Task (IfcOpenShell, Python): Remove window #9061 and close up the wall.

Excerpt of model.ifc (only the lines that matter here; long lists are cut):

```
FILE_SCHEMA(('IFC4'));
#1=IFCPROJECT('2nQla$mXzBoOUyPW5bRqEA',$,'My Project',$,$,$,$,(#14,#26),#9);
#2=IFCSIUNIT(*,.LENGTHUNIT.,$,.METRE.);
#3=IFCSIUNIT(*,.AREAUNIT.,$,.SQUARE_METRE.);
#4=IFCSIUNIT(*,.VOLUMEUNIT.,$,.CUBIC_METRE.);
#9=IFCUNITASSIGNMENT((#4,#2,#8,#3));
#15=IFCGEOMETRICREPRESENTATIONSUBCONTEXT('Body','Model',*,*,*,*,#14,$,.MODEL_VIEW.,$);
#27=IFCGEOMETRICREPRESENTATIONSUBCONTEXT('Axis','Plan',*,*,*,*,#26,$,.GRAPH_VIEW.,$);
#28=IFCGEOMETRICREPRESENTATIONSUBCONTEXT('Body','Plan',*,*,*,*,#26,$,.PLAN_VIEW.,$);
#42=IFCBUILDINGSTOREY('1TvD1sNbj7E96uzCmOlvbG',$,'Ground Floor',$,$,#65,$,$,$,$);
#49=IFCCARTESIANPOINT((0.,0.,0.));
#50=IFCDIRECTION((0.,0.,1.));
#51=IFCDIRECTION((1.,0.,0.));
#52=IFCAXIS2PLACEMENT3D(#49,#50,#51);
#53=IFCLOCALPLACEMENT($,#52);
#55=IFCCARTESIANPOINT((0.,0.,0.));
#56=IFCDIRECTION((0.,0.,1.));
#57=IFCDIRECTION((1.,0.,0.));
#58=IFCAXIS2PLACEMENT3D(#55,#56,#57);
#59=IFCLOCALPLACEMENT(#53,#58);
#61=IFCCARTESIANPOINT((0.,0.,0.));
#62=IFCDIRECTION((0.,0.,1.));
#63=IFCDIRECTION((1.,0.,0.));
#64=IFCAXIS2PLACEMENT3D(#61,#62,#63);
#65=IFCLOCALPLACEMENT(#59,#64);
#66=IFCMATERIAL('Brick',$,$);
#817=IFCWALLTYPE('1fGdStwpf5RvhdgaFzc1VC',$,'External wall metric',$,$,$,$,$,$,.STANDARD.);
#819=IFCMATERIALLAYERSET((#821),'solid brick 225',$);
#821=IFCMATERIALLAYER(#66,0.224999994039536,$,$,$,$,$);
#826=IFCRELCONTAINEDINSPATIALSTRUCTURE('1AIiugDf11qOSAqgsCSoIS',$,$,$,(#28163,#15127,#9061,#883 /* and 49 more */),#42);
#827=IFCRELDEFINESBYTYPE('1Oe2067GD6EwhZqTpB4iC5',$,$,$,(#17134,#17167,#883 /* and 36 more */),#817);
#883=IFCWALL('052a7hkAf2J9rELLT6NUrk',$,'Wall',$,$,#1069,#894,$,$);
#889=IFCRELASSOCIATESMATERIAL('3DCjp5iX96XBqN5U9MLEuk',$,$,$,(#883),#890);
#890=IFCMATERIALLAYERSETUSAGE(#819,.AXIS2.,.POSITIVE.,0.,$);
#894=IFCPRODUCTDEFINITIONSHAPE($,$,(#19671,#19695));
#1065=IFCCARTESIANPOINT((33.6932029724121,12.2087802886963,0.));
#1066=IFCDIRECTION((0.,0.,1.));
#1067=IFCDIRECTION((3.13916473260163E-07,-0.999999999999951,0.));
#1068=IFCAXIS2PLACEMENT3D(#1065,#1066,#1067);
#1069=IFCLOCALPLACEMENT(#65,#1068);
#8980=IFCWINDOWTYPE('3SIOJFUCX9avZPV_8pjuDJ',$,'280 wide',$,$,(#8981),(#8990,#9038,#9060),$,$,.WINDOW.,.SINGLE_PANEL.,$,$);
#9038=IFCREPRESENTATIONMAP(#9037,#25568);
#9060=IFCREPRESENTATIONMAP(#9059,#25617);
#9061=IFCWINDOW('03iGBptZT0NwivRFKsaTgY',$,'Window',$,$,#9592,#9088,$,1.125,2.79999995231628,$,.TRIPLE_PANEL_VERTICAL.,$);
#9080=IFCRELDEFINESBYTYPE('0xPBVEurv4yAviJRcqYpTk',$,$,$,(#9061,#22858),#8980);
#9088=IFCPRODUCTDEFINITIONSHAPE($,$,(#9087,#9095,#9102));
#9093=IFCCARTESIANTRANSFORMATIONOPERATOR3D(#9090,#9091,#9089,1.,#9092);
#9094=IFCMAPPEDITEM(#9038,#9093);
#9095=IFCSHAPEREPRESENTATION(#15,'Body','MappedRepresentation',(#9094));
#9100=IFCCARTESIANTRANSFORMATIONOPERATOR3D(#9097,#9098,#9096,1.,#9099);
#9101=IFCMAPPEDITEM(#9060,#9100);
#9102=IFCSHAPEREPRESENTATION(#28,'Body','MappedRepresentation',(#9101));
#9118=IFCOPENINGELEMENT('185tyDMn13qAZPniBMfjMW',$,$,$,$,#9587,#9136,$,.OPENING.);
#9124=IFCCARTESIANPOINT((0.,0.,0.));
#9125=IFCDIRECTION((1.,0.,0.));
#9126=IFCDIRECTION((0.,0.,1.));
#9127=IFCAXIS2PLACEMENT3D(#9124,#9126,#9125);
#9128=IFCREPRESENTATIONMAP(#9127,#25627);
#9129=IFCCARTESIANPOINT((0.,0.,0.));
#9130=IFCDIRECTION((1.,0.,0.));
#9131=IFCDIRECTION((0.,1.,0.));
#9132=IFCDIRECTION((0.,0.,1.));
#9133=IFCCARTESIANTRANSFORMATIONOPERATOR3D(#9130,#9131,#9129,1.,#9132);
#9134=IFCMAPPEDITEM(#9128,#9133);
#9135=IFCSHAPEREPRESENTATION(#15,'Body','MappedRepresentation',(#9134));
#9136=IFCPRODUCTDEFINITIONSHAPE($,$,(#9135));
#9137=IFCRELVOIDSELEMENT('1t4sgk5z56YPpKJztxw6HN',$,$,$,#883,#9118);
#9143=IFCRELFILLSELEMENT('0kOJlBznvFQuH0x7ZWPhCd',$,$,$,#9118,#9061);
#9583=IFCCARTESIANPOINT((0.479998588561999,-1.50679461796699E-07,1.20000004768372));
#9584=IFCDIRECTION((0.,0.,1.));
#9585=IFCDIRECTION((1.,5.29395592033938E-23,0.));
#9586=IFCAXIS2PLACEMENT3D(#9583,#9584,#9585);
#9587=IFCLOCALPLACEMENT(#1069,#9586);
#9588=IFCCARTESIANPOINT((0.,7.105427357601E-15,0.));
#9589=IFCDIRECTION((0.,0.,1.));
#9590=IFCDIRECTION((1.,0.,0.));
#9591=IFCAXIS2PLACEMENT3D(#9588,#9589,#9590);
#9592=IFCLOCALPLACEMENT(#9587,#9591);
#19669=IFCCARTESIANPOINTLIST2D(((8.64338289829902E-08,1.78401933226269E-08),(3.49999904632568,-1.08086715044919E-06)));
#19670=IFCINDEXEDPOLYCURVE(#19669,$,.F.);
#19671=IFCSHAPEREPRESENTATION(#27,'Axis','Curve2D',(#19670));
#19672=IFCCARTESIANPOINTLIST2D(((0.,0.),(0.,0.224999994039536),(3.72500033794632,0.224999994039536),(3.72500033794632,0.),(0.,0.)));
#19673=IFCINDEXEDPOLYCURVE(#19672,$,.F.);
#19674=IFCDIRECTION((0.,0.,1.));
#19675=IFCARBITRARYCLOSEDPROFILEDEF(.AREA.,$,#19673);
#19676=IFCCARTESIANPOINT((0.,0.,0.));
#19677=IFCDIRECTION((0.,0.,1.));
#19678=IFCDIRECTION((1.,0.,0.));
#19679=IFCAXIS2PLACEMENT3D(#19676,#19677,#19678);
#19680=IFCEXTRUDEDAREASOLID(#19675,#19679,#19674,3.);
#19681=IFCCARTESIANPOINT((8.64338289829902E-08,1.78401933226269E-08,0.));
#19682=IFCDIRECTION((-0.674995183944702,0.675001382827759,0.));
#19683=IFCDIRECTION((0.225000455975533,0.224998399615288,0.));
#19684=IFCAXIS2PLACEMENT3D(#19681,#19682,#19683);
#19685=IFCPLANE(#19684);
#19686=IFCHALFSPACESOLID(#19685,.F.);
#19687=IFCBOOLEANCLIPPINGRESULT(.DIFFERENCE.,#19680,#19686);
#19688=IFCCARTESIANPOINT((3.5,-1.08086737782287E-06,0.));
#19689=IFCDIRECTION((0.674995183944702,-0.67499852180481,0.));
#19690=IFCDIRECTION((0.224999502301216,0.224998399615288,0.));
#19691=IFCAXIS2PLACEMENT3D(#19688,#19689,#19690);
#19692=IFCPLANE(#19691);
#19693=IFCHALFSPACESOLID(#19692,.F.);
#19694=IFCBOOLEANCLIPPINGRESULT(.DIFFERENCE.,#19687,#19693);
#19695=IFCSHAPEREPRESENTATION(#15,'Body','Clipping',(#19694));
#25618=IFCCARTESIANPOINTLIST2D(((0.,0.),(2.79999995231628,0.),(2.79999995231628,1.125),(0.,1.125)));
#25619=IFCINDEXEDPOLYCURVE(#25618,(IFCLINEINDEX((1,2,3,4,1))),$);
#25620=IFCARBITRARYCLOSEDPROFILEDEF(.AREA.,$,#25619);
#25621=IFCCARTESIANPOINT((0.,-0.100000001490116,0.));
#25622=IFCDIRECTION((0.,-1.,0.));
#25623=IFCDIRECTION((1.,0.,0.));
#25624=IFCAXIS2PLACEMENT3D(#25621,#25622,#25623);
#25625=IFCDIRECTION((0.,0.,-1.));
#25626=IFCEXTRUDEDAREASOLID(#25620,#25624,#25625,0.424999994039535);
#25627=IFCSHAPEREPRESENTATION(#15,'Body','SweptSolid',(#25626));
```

```python
import ifcopenshell
import ifcopenshell.api.feature
import ifcopenshell.api.root
import ifcopenshell.geom
import ifcopenshell.util.shape

model = ifcopenshell.open("model.ifc")
settings = ifcopenshell.geom.settings()


def volume(element):
    """Net volume in cubic metres, openings subtracted."""
    shape = ifcopenshell.geom.create_shape(settings, element)
    return ifcopenshell.util.shape.get_volume(shape.geometry)


window = model.by_guid("03iGBptZT0NwivRFKsaTgY")
opening = window.FillsVoids[0].RelatingOpeningElement
wall = opening.VoidsElements[0].RelatingBuildingElement
before = volume(wall)

ifcopenshell.api.root.remove_product(model, product=window)
ifcopenshell.api.feature.remove_feature(model, feature=opening)

after = volume(wall)

print(f"wall volume {before:.3f} -> {after:.3f} m3")

model.write("model_v2.ifc")
```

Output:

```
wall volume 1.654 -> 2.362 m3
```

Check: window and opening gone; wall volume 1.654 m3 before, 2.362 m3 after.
